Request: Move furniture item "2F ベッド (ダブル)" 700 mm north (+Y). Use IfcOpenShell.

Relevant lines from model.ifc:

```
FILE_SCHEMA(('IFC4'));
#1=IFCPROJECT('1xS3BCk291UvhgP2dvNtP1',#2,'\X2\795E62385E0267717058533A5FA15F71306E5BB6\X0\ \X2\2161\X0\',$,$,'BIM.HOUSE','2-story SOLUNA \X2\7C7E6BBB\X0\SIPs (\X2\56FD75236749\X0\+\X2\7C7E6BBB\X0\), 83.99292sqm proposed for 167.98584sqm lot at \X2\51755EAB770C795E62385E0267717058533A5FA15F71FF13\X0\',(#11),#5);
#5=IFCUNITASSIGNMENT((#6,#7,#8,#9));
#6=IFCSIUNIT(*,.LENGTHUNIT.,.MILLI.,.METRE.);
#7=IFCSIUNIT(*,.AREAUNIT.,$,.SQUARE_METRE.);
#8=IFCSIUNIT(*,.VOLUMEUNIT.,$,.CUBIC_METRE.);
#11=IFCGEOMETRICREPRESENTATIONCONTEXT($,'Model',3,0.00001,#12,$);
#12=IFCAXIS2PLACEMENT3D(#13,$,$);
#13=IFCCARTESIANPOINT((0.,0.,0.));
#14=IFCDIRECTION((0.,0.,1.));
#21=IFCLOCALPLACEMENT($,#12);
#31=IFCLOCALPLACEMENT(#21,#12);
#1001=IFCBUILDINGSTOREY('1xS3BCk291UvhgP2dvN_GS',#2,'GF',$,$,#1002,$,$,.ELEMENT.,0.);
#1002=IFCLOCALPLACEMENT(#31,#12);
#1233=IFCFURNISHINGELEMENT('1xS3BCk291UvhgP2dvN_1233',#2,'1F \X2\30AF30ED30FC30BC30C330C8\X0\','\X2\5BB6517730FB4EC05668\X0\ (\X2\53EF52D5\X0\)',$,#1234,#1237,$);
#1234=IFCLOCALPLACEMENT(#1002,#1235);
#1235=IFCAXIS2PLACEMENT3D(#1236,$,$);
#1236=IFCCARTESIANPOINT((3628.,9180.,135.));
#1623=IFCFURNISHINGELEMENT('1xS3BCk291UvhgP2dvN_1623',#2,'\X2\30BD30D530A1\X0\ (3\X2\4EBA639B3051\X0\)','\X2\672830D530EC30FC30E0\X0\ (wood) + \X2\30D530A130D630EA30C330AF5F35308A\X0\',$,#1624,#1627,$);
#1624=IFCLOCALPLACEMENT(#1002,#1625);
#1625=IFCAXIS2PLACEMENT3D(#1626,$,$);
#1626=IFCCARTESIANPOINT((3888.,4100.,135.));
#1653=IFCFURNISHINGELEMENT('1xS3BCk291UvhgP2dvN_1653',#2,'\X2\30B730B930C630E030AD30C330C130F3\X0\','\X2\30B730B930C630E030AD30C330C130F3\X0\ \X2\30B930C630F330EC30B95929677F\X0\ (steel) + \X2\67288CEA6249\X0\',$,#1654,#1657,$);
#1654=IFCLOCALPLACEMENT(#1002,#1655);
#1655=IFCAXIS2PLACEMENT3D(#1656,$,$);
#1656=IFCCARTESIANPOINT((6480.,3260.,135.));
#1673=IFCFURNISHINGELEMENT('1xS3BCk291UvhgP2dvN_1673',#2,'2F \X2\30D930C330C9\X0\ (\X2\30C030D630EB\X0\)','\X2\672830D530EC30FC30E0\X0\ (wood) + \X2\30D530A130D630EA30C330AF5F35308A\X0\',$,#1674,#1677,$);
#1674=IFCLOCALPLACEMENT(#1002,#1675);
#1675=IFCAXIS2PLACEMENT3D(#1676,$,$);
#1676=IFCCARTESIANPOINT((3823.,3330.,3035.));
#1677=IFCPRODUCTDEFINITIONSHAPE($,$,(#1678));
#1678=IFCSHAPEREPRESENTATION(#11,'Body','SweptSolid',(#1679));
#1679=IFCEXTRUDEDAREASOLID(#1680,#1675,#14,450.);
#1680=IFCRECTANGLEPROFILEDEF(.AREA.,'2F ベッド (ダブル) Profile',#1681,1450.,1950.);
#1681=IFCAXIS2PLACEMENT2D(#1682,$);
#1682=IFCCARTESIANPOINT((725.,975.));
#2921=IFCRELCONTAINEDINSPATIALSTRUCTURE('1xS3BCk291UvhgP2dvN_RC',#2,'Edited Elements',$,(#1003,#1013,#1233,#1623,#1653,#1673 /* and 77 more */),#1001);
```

```python
import ifcopenshell
import ifcopenshell.api.geometry
import ifcopenshell.util.placement
import ifcopenshell.util.unit

model = ifcopenshell.open("model.ifc")
unit_scale = ifcopenshell.util.unit.calculate_unit_scale(model)

item = model.by_guid("1xS3BCk291UvhgP2dvN_1673")
matrix = ifcopenshell.util.placement.get_local_placement(item.ObjectPlacement)
matrix[1, 3] += 0.7 / unit_scale
ifcopenshell.api.geometry.edit_object_placement(model, product=item, matrix=matrix, is_si=False)

print(ifcopenshell.util.placement.get_local_placement(item.ObjectPlacement).round(3) + 0.0)

model.write("model-out.ifc")
```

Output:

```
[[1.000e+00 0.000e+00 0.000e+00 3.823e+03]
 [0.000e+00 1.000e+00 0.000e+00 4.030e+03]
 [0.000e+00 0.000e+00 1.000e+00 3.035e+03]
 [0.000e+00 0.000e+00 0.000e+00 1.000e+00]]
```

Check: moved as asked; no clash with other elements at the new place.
